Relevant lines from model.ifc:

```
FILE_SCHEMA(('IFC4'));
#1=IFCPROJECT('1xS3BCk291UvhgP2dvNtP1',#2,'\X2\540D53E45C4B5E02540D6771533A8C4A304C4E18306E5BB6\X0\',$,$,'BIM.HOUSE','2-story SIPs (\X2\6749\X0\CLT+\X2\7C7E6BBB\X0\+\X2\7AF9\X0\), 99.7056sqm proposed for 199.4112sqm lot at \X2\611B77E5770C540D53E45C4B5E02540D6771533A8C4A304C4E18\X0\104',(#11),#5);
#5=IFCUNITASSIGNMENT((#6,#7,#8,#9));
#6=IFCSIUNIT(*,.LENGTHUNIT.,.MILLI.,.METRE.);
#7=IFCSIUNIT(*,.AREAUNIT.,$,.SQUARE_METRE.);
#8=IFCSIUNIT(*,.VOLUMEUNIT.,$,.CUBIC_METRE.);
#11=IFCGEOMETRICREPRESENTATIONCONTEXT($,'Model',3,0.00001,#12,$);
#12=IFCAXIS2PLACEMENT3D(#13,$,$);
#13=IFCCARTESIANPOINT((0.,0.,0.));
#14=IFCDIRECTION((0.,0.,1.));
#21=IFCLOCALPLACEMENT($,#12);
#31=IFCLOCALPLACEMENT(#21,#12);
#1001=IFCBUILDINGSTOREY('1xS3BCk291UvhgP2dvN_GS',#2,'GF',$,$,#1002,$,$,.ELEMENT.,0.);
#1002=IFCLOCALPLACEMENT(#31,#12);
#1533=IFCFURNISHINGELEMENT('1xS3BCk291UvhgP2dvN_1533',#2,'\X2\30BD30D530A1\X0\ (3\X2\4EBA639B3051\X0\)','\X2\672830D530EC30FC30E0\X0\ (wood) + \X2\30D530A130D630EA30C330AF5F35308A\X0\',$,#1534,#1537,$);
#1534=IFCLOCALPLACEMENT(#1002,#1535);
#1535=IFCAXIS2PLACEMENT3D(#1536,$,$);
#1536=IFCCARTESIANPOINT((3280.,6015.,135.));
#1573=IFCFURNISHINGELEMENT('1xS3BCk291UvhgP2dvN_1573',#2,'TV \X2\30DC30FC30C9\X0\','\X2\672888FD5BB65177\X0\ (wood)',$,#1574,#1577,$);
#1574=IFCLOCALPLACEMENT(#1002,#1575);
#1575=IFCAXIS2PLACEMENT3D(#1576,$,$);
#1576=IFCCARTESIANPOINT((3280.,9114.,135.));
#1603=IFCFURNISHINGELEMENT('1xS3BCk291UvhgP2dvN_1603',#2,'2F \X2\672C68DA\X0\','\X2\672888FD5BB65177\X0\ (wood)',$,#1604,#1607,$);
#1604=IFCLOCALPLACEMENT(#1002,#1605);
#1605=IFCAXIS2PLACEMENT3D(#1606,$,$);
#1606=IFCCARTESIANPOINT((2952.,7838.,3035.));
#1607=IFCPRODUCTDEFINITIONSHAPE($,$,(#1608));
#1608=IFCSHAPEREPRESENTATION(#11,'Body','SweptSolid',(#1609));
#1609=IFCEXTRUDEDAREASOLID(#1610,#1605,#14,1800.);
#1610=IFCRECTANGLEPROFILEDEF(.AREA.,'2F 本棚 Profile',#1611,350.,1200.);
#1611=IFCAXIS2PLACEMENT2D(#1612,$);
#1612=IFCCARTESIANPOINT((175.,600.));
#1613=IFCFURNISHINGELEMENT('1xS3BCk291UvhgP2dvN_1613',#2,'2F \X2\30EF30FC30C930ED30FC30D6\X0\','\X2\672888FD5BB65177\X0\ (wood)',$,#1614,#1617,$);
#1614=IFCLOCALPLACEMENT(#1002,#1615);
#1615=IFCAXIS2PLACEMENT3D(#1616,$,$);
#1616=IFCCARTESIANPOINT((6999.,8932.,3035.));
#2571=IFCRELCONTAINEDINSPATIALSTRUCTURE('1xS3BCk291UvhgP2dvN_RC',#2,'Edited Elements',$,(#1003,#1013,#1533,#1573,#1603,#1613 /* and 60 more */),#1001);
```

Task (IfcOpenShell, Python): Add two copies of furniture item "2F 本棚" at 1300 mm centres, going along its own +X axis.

```python
import ifcopenshell
import ifcopenshell.api.geometry
import ifcopenshell.api.root
import ifcopenshell.util.element
import ifcopenshell.util.placement

model = ifcopenshell.open("model.ifc")


def reuse_history(source, copy):
    """copy_class also copies each property set's owner history, people and application; keep the originals."""
    for rel in copy.IsDefinedBy:
        if rel.is_a("IfcRelDefinesByProperties") and (history := rel.RelatingPropertyDefinition.OwnerHistory):
            rel.RelatingPropertyDefinition.OwnerHistory = source.OwnerHistory
            ifcopenshell.util.element.remove_deep2(model, history)


source = model.by_guid("1xS3BCk291UvhgP2dvN_1603")
base = ifcopenshell.util.placement.get_local_placement(source.ObjectPlacement)
step = base[:3, 0] * 1300.0

for i in range(1, 3):
    copy = ifcopenshell.api.root.copy_class(model, product=source)
    copy.Representation = ifcopenshell.util.element.copy_deep(
        model, source.Representation, exclude=["IfcGeometricRepresentationContext", "IfcRepresentationMap"]
    )
    reuse_history(source, copy)
    matrix = base.copy()
    matrix[:3, 3] += i * step
    print("added at", matrix[:3, 3].round(3) + 0.0)
    ifcopenshell.api.geometry.edit_object_placement(model, product=copy, matrix=matrix, is_si=False)

model.write("model_rev.ifc")
```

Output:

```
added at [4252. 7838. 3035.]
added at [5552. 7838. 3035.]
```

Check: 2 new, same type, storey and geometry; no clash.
